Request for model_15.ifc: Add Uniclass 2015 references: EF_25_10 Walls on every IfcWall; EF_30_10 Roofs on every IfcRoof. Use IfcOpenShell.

First a look at what the model holds.

```python
import ifcopenshell

model = ifcopenshell.open("model_15.ifc")
print(model.schema)
print("classifications:", [c.Name for c in model.by_type("IfcClassification")])
for ifc_class in ("IfcDoor", "IfcRoof", "IfcStair", "IfcWall", "IfcWindow"):
    print(ifc_class, len(model.by_type(ifc_class)))
```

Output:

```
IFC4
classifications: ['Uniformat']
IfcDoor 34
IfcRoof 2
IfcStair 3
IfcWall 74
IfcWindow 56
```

```python
import ifcopenshell
import ifcopenshell.api.classification

model = ifcopenshell.open("model_15.ifc")

system = ifcopenshell.api.classification.add_classification(model, classification="Uniclass 2015")

codes = {
    "IfcWall": ("EF_25_10", "Walls"),
    "IfcRoof": ("EF_30_10", "Roofs"),
}
for ifc_class, (code, name) in codes.items():
    products = model.by_type(ifc_class)
    ifcopenshell.api.classification.add_reference(
        model, products=products, classification=system, identification=code, name=name
    )
    print(code, len(products))

model.write("model_15_rev.ifc")
```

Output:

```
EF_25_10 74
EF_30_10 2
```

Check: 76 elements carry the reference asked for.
